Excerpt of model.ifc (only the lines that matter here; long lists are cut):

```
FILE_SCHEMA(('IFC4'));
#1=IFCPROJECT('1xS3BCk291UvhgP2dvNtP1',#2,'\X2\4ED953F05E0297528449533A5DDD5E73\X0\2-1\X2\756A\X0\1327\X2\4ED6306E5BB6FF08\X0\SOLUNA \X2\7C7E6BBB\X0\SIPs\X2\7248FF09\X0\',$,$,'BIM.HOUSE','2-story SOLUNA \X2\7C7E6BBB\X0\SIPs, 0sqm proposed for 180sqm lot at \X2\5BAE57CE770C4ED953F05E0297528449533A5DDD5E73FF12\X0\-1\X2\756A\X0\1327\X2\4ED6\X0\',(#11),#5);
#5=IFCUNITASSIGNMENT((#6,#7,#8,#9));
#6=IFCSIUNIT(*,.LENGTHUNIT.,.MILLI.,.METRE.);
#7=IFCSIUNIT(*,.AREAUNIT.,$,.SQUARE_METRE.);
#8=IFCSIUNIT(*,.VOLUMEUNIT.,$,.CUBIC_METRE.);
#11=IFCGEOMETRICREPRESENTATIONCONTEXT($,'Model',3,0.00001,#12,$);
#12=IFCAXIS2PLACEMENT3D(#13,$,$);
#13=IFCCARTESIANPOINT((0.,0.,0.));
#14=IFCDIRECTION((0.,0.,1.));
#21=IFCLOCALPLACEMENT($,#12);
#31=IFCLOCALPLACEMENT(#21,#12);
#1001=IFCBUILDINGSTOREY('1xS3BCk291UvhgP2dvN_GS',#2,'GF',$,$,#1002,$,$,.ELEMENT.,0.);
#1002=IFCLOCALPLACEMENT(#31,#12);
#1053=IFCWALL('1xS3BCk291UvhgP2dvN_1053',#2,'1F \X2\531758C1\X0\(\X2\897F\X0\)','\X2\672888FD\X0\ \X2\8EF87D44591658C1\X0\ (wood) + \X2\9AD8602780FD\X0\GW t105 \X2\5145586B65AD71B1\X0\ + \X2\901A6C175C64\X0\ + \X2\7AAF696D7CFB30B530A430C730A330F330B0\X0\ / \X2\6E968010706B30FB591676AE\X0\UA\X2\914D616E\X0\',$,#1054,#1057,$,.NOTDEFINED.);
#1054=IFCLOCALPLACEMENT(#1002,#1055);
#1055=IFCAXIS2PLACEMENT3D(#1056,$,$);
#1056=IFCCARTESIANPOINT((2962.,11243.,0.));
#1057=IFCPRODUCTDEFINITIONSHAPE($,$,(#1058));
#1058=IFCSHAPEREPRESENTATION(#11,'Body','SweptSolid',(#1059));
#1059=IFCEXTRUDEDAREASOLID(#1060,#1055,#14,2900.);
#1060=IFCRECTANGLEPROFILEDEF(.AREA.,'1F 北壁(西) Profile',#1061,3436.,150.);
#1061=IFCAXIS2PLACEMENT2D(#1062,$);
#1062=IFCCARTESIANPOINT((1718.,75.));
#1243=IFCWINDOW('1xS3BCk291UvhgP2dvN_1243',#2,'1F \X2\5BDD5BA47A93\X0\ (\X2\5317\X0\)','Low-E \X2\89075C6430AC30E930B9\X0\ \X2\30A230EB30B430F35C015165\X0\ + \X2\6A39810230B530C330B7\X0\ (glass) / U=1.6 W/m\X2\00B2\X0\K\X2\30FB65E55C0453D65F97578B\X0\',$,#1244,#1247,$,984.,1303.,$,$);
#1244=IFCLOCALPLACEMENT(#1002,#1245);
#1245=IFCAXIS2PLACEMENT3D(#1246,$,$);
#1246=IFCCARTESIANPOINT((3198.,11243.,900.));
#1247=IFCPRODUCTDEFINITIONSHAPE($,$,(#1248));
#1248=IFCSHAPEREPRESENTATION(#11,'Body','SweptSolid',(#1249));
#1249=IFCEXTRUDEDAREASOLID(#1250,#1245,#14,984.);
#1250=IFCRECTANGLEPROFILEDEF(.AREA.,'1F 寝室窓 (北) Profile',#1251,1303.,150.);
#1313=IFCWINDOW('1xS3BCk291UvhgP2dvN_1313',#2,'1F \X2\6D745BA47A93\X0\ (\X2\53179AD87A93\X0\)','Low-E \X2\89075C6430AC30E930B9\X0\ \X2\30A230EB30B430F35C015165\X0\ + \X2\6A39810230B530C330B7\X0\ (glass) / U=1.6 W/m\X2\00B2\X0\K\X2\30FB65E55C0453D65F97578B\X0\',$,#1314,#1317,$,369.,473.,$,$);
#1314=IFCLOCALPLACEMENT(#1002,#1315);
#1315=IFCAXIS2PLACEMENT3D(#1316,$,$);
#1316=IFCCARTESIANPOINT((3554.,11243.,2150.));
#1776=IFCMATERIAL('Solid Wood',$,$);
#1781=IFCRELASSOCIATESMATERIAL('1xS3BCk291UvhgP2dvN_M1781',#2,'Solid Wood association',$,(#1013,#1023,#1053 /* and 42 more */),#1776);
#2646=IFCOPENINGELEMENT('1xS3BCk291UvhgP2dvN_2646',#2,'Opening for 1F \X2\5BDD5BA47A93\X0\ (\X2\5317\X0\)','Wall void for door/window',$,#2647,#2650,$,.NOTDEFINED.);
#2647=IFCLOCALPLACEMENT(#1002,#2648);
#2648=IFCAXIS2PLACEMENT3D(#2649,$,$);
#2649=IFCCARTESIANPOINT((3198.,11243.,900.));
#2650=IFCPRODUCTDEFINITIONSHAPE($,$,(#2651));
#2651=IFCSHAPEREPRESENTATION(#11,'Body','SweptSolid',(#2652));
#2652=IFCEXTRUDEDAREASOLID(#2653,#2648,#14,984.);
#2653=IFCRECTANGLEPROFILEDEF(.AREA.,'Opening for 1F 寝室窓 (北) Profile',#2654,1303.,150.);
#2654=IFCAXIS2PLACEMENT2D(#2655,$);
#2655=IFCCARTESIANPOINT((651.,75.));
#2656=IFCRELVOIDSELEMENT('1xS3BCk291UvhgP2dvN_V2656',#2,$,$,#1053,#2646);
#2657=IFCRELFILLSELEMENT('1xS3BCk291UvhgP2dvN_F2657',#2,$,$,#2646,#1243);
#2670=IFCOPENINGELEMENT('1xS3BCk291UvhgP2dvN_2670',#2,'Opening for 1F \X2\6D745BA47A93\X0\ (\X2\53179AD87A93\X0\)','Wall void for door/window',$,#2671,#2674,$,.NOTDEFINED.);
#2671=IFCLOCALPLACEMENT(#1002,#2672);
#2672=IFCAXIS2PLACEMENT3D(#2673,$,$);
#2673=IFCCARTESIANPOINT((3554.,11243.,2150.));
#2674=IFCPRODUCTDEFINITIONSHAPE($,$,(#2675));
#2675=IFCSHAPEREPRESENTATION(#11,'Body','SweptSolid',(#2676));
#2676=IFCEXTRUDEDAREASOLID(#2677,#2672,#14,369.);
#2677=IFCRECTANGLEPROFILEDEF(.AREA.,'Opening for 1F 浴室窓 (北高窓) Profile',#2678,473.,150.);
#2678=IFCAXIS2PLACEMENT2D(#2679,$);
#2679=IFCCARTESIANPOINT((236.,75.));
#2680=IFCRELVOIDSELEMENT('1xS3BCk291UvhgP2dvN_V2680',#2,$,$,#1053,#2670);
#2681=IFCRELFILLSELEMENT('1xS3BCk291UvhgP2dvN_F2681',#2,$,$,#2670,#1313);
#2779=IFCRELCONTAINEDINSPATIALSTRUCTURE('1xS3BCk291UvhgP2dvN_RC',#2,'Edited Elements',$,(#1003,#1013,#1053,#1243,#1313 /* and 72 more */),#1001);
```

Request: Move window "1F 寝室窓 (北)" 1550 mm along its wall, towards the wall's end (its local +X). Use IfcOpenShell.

```python
import ifcopenshell
import ifcopenshell.api.geometry
import ifcopenshell.util.placement
import ifcopenshell.util.unit

model = ifcopenshell.open("model.ifc")
unit_scale = ifcopenshell.util.unit.calculate_unit_scale(model)

window = model.by_guid("1xS3BCk291UvhgP2dvN_1243")
opening = window.FillsVoids[0].RelatingOpeningElement
wall = opening.VoidsElements[0].RelatingBuildingElement

wall_matrix = ifcopenshell.util.placement.get_local_placement(wall.ObjectPlacement)
shift = wall_matrix[:3, 0] * 1.55 / unit_scale
before = ifcopenshell.util.placement.get_local_placement(window.ObjectPlacement)[:3, 3].copy()

# The window is not placed relative to its opening, so move both.
for product in (opening, window):
    matrix = ifcopenshell.util.placement.get_local_placement(product.ObjectPlacement)
    matrix[:3, 3] += shift
    ifcopenshell.api.geometry.edit_object_placement(model, product=product, matrix=matrix, is_si=False)

after = ifcopenshell.util.placement.get_local_placement(window.ObjectPlacement)[:3, 3]
print("window moved by", (after - before).round(3) + 0.0)

model.write("model_updated.ifc")
```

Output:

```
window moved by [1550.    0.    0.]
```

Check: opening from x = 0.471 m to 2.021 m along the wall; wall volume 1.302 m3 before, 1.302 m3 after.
